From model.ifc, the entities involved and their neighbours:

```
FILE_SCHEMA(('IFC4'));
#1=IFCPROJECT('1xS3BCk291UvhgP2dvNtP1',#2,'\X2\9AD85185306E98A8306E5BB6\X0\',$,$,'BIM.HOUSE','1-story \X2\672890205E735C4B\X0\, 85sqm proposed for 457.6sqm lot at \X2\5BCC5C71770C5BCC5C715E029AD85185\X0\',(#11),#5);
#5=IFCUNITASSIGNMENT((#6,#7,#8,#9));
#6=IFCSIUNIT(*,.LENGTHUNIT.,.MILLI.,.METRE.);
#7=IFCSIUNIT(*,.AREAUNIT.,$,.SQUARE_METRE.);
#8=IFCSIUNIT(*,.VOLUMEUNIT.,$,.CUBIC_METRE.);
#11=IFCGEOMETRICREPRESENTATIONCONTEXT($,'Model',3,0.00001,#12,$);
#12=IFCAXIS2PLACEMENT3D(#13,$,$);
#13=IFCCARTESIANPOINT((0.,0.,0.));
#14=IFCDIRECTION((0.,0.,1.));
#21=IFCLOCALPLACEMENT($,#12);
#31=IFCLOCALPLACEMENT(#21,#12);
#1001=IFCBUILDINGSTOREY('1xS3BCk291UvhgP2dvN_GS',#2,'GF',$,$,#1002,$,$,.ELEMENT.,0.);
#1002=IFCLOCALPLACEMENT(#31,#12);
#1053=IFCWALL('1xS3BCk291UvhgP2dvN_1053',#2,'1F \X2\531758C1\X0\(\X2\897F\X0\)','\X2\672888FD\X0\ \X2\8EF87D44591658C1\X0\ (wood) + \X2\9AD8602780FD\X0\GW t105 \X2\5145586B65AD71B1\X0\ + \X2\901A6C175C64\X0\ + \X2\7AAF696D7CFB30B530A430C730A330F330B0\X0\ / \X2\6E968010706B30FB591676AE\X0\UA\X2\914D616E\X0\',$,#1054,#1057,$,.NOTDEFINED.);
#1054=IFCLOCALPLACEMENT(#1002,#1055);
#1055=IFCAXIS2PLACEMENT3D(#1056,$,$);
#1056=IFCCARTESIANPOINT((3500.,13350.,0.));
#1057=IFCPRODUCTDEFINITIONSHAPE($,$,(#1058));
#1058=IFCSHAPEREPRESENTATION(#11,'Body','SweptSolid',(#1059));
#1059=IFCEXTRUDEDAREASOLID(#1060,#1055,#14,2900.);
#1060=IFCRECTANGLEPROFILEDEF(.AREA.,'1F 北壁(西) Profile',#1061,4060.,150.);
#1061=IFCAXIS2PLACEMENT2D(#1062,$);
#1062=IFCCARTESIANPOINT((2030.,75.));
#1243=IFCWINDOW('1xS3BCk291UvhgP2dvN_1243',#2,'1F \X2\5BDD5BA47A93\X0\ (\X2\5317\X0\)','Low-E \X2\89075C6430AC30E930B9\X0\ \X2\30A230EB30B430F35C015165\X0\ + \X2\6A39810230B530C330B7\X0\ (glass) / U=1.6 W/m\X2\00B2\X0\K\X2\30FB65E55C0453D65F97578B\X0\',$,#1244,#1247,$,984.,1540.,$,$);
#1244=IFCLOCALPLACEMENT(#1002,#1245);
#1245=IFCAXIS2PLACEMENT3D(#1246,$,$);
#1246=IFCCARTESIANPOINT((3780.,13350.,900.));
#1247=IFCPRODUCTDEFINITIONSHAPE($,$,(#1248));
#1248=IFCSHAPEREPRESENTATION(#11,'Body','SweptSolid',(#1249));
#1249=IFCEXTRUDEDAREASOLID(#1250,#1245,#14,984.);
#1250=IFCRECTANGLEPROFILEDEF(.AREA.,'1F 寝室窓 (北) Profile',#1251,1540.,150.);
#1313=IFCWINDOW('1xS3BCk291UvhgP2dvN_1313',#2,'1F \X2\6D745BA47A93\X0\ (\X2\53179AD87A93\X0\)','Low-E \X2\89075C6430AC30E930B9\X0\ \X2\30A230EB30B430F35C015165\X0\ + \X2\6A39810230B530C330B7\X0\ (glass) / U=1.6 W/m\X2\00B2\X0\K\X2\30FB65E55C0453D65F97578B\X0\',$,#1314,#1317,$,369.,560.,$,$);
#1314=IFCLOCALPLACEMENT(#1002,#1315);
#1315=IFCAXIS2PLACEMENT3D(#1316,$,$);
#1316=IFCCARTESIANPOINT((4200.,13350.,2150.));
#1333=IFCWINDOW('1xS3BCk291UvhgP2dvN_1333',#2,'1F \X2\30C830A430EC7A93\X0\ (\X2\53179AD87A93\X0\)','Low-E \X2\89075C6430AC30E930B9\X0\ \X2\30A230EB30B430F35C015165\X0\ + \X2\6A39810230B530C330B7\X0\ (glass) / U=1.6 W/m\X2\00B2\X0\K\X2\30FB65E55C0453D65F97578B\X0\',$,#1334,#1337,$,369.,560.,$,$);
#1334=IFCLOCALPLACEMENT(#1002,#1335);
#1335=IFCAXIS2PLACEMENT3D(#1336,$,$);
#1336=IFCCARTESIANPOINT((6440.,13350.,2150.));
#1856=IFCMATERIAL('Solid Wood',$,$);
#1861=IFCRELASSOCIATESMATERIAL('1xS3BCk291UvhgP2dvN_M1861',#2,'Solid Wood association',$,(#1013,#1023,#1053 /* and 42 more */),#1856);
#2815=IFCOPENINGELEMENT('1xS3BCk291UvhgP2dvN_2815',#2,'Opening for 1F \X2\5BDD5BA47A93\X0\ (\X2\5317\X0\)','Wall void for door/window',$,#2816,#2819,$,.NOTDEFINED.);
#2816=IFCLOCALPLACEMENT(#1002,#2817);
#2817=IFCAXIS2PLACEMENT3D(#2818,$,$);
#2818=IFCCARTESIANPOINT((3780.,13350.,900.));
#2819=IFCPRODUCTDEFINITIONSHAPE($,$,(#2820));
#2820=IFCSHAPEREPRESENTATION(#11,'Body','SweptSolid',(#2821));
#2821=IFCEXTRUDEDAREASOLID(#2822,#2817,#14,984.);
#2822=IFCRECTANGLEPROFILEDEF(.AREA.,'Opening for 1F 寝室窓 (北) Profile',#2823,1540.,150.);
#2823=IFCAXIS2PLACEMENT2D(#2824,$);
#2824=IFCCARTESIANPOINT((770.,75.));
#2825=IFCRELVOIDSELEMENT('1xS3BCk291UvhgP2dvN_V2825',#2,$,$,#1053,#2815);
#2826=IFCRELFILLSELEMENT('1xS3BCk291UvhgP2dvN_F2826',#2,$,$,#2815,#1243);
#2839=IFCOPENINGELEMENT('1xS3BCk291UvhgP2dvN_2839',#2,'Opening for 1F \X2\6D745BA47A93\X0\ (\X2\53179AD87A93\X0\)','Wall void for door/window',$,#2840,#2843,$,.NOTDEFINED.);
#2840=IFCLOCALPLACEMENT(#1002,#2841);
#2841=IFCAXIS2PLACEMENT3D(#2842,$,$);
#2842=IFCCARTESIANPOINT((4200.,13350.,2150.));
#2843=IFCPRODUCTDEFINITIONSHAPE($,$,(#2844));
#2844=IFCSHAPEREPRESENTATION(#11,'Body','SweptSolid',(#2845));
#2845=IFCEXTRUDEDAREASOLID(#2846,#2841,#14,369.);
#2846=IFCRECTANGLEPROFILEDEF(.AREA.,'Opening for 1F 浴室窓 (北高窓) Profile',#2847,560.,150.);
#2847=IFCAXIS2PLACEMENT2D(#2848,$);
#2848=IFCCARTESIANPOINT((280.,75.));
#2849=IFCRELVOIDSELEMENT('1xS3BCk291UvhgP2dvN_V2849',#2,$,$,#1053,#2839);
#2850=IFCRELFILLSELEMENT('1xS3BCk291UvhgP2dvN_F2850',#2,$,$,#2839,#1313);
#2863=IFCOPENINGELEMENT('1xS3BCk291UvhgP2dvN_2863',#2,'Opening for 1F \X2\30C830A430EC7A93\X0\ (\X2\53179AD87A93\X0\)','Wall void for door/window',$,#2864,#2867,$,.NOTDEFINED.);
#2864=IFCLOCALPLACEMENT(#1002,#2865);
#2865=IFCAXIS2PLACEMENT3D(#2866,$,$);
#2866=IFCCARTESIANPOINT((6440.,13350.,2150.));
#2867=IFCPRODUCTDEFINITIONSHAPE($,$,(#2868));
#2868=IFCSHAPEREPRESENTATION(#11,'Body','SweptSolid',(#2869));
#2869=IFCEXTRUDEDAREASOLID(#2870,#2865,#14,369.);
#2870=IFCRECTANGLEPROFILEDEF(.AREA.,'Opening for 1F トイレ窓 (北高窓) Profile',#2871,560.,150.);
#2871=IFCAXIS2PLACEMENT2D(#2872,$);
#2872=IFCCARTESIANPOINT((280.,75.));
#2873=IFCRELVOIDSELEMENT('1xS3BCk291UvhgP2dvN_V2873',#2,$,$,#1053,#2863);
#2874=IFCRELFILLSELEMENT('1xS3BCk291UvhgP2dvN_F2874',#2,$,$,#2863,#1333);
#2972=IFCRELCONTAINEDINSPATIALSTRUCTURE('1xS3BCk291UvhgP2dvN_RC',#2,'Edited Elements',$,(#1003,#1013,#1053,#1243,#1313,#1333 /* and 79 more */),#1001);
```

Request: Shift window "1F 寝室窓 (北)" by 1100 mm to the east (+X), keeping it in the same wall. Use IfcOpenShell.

```python
import ifcopenshell
import ifcopenshell.api.geometry
import ifcopenshell.util.placement

model = ifcopenshell.open("model.ifc")

window = model.by_guid("1xS3BCk291UvhgP2dvN_1243")
opening = window.FillsVoids[0].RelatingOpeningElement
wall = opening.VoidsElements[0].RelatingBuildingElement

wall_matrix = ifcopenshell.util.placement.get_local_placement(wall.ObjectPlacement)
shift = wall_matrix[:3, 0] * 1100.0
before = ifcopenshell.util.placement.get_local_placement(window.ObjectPlacement)[:3, 3].copy()

# The window is not placed relative to its opening, so move both.
for product in (opening, window):
    matrix = ifcopenshell.util.placement.get_local_placement(product.ObjectPlacement)
    matrix[:3, 3] += shift
    ifcopenshell.api.geometry.edit_object_placement(model, product=product, matrix=matrix, is_si=False)

after = ifcopenshell.util.placement.get_local_placement(window.ObjectPlacement)[:3, 3]
print("window moved by", (after - before).round(3) + 0.0)

model.write("model-out.ifc")
```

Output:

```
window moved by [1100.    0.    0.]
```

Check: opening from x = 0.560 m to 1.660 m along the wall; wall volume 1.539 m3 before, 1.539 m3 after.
